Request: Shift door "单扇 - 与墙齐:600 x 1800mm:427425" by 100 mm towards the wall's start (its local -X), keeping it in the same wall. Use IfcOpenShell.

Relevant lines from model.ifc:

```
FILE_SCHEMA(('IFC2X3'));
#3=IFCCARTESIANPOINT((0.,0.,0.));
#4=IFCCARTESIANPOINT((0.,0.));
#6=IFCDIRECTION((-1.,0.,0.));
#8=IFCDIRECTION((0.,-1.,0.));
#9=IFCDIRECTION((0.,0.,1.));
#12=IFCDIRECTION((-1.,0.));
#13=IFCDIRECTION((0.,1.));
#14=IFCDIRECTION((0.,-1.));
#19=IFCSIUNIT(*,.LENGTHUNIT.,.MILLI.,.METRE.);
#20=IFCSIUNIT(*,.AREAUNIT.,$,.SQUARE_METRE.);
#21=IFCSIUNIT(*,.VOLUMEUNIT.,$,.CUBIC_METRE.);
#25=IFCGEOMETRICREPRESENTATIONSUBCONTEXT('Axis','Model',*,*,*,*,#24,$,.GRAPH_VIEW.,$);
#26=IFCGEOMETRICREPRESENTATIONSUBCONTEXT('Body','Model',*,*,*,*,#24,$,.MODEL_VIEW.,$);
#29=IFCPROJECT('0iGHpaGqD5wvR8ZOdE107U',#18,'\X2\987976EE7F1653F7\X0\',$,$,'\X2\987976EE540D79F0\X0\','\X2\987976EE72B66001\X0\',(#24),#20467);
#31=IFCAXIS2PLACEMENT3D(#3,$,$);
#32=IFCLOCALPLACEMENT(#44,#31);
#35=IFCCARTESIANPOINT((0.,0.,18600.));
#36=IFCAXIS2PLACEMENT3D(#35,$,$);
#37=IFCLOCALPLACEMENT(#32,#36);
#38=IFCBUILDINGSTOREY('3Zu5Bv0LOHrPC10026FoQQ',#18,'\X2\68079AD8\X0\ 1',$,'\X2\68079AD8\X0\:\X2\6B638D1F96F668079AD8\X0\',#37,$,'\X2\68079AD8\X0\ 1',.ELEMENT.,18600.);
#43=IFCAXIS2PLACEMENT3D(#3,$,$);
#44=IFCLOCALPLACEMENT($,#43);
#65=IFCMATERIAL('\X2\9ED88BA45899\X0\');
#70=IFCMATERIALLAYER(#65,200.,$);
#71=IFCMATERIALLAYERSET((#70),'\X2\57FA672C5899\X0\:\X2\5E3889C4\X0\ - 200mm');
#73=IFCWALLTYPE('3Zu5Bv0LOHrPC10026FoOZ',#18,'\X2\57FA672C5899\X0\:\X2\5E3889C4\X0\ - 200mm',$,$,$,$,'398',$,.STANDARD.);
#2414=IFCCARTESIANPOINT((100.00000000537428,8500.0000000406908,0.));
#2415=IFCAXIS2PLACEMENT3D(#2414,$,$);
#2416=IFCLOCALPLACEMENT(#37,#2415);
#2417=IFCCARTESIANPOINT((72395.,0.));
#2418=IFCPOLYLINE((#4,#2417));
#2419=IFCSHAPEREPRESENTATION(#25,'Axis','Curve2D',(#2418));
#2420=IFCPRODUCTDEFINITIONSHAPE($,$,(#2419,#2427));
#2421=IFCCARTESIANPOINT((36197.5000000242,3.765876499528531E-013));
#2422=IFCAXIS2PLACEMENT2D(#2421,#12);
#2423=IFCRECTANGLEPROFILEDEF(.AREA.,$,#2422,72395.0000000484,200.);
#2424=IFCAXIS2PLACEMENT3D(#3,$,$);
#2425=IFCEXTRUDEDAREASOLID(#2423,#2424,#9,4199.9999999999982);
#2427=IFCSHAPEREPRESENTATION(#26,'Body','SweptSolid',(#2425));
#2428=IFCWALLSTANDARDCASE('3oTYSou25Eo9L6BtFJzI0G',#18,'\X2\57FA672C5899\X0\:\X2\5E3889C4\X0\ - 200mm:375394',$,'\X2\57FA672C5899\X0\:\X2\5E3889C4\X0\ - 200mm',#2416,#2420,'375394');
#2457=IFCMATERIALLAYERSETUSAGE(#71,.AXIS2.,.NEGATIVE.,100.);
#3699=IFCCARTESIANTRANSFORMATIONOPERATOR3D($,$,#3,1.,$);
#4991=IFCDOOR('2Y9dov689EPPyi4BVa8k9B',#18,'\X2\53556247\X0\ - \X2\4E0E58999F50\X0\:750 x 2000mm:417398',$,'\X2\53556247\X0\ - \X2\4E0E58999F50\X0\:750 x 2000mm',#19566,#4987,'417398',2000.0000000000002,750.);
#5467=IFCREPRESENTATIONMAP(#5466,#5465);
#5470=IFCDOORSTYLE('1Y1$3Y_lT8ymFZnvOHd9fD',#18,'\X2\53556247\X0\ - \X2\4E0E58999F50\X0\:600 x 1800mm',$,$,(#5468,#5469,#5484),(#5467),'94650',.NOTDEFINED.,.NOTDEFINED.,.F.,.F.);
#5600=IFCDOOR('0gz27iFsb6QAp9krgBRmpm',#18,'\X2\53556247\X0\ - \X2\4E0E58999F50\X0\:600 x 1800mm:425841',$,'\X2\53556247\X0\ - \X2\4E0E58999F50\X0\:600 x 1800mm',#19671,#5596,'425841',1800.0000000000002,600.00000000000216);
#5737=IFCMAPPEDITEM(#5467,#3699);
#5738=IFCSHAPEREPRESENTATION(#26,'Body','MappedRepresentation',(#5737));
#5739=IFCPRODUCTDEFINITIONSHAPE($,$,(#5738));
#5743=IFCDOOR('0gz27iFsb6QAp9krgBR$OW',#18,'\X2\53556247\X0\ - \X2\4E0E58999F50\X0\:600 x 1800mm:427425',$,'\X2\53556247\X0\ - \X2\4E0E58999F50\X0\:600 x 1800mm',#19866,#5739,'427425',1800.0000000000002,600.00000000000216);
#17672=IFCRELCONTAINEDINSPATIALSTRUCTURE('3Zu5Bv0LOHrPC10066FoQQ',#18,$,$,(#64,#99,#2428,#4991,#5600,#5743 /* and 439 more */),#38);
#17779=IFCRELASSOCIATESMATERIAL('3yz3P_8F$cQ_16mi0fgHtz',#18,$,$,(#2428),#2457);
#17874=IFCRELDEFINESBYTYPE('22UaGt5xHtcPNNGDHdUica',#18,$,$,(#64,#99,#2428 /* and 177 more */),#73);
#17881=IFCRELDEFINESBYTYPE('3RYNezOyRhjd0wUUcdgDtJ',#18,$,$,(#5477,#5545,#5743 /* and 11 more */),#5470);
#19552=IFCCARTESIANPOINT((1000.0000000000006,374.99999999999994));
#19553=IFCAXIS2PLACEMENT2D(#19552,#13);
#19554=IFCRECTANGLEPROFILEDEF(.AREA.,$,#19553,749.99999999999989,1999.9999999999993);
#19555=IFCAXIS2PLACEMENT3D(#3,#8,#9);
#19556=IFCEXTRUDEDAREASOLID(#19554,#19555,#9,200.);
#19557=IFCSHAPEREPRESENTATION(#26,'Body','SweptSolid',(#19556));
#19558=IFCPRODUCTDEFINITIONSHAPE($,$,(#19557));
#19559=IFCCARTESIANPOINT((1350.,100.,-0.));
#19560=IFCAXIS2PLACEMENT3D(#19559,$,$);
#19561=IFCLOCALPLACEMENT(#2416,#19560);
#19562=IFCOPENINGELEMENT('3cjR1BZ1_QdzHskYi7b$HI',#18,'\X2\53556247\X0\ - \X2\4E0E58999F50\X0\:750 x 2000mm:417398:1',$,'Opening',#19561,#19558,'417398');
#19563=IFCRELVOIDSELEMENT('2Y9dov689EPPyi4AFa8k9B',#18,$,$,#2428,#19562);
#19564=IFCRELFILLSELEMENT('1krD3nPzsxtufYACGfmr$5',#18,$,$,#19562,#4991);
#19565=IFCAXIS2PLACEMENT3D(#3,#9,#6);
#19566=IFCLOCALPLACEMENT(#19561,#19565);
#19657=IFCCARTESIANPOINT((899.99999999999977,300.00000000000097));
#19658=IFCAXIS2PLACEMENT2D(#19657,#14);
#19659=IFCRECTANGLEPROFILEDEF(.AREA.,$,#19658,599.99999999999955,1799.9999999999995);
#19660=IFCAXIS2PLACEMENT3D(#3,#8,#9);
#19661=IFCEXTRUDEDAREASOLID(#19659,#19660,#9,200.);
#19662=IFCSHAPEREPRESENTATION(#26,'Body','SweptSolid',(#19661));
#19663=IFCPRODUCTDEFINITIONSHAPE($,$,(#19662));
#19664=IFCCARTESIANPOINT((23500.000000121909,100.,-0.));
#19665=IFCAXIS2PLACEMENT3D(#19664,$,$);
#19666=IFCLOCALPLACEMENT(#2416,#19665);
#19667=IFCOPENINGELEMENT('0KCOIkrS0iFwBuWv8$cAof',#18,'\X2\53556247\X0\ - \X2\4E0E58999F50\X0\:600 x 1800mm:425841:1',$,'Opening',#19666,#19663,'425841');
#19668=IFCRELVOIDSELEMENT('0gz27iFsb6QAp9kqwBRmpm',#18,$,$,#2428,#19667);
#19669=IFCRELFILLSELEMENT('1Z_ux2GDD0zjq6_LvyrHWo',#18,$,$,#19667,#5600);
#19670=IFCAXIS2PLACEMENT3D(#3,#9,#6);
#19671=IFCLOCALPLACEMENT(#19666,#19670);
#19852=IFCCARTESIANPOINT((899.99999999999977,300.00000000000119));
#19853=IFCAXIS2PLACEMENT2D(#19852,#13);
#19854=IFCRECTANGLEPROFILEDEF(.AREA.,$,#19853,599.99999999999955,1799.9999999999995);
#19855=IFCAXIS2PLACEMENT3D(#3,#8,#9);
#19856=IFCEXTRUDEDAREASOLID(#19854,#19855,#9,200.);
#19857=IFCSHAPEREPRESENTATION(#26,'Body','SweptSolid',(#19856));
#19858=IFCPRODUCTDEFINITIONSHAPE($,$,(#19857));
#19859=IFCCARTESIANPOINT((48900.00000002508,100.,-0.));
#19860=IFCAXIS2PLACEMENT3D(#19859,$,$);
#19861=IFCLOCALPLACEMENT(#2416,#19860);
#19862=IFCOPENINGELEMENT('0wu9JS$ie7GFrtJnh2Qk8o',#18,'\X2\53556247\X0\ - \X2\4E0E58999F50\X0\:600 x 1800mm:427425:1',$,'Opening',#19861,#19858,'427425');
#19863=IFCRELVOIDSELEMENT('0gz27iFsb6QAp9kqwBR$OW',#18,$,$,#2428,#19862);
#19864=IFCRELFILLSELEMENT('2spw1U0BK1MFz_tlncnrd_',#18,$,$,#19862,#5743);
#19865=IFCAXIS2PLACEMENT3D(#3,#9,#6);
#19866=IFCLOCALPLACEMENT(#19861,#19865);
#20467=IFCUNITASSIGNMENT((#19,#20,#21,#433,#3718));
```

```python
import ifcopenshell
import ifcopenshell.api.geometry
import ifcopenshell.util.placement
import ifcopenshell.util.unit

model = ifcopenshell.open("model.ifc")
unit_scale = ifcopenshell.util.unit.calculate_unit_scale(model)

door = model.by_guid("0gz27iFsb6QAp9krgBR$OW")
opening = door.FillsVoids[0].RelatingOpeningElement
wall = opening.VoidsElements[0].RelatingBuildingElement

wall_matrix = ifcopenshell.util.placement.get_local_placement(wall.ObjectPlacement)
shift = wall_matrix[:3, 0] * -0.1 / unit_scale
before = ifcopenshell.util.placement.get_local_placement(door.ObjectPlacement)[:3, 3].copy()

# The door is placed relative to its opening, so it follows when the opening moves.
matrix = ifcopenshell.util.placement.get_local_placement(opening.ObjectPlacement)
matrix[:3, 3] += shift
ifcopenshell.api.geometry.edit_object_placement(
    model, product=opening, matrix=matrix, is_si=False, should_transform_children=True
)

after = ifcopenshell.util.placement.get_local_placement(door.ObjectPlacement)[:3, 3]
print("door moved by", (after - before).round(3) + 0.0)

model.write("model_edited.ifc")
```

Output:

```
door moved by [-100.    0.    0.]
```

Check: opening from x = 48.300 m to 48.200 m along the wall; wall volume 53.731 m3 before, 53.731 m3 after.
